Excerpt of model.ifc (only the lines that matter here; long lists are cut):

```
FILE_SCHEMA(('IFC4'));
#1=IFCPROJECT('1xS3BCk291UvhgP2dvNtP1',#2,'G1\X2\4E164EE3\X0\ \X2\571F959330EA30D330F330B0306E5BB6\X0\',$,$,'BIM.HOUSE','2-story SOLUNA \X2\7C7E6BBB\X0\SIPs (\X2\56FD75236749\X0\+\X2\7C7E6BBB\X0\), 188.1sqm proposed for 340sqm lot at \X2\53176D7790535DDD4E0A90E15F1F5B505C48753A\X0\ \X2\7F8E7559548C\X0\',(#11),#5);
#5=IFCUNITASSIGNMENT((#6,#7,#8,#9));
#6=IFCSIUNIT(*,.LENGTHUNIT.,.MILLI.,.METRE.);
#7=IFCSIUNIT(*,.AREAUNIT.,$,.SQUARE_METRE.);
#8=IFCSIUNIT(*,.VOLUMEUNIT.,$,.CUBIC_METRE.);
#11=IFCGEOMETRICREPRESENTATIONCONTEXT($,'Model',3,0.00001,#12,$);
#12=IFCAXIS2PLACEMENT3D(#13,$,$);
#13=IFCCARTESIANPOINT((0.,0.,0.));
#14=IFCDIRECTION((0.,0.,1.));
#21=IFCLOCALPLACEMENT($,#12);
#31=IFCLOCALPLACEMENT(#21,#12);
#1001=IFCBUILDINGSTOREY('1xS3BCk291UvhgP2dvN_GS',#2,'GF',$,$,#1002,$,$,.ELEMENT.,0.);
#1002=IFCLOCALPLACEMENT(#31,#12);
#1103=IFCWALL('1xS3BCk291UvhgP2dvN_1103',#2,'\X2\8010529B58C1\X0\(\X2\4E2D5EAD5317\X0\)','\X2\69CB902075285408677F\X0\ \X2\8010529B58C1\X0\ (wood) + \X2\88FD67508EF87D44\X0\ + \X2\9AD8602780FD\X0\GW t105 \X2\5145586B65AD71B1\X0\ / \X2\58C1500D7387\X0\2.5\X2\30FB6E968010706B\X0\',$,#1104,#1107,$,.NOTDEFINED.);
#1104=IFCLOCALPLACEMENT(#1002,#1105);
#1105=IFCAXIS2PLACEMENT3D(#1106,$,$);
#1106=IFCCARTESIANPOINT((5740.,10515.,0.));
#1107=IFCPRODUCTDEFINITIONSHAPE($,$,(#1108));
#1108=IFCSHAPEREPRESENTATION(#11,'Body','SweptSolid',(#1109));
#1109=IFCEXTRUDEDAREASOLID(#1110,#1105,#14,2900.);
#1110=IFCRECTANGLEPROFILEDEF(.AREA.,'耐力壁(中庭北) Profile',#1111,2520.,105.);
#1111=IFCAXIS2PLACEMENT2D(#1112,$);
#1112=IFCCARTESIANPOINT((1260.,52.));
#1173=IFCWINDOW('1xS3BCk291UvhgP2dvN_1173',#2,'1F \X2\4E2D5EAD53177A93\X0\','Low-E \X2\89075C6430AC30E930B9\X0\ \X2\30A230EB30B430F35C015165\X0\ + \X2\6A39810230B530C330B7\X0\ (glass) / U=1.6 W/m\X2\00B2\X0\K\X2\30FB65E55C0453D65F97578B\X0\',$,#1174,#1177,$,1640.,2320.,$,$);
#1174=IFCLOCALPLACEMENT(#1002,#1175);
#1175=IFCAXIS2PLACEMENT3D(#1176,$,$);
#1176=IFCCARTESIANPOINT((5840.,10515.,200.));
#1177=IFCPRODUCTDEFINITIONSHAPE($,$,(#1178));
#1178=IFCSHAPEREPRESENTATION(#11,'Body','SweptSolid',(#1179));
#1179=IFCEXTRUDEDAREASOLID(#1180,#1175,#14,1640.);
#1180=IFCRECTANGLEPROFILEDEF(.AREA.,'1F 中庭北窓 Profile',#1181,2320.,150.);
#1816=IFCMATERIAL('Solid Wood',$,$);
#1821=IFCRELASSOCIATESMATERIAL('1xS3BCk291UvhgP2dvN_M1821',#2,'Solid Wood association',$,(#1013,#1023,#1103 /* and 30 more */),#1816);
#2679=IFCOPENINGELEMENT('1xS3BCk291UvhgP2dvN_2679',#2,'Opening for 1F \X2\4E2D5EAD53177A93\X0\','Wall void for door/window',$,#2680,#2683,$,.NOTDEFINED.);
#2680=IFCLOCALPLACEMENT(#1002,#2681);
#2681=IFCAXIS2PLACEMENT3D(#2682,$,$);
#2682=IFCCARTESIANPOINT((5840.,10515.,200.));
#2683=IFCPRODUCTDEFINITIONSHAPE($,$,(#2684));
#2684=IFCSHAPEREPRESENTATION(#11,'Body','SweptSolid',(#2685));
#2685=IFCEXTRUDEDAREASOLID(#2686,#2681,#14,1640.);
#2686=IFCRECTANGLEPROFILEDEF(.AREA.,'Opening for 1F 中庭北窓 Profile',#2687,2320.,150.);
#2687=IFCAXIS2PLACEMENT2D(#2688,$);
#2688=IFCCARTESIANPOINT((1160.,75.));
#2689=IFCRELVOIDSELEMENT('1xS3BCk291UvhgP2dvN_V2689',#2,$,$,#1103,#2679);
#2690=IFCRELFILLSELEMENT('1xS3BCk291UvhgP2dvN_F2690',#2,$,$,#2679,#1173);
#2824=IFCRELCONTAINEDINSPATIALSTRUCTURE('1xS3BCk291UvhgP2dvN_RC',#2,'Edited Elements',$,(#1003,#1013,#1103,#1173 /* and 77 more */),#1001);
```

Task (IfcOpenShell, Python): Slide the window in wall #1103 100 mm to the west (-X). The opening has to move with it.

```python
import ifcopenshell
import ifcopenshell.api.geometry
import ifcopenshell.util.placement
import ifcopenshell.util.unit

model = ifcopenshell.open("model.ifc")
unit_scale = ifcopenshell.util.unit.calculate_unit_scale(model)

window = model.by_id(1173)
opening = window.FillsVoids[0].RelatingOpeningElement
wall = opening.VoidsElements[0].RelatingBuildingElement

wall_matrix = ifcopenshell.util.placement.get_local_placement(wall.ObjectPlacement)
shift = wall_matrix[:3, 0] * -0.1 / unit_scale
before = ifcopenshell.util.placement.get_local_placement(window.ObjectPlacement)[:3, 3].copy()

# The window is not placed relative to its opening, so move both.
for product in (opening, window):
    matrix = ifcopenshell.util.placement.get_local_placement(product.ObjectPlacement)
    matrix[:3, 3] += shift
    ifcopenshell.api.geometry.edit_object_placement(model, product=product, matrix=matrix, is_si=False)

after = ifcopenshell.util.placement.get_local_placement(window.ObjectPlacement)[:3, 3]
print("window moved by", (after - before).round(3) + 0.0)

model.write("model_edited.ifc")
```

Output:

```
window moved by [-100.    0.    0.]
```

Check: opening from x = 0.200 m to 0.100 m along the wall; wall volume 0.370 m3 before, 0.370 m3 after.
